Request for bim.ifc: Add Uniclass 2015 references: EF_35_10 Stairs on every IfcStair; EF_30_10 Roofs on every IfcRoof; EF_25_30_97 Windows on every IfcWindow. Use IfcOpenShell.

First a look at what the model holds.

```python
import ifcopenshell

model = ifcopenshell.open("bim.ifc")
print(model.schema)
print("classifications:", [c.Name for c in model.by_type("IfcClassification")])
for ifc_class in ("IfcDoor", "IfcRoof", "IfcStair", "IfcWall", "IfcWindow"):
    print(ifc_class, len(model.by_type(ifc_class)))
```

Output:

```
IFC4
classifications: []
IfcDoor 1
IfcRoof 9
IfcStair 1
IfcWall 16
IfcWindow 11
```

```python
import ifcopenshell
import ifcopenshell.api.classification

model = ifcopenshell.open("bim.ifc")

system = ifcopenshell.api.classification.add_classification(model, classification="Uniclass 2015")

codes = {
    "IfcStair": ("EF_35_10", "Stairs"),
    "IfcRoof": ("EF_30_10", "Roofs"),
    "IfcWindow": ("EF_25_30_97", "Windows"),
}
for ifc_class, (code, name) in codes.items():
    products = model.by_type(ifc_class)
    ifcopenshell.api.classification.add_reference(
        model, products=products, classification=system, identification=code, name=name
    )
    print(code, len(products))

model.write("bim-out.ifc")
```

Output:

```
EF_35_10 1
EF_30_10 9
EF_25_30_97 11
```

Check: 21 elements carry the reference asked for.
